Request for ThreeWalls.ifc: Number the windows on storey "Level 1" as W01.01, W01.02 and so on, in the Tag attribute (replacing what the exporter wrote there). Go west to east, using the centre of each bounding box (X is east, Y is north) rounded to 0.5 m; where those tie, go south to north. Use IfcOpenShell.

First a look at what the model holds.

```python
import ifcopenshell
import ifcopenshell.util.element
import ifcopenshell.util.placement

model = ifcopenshell.open("ThreeWalls.ifc")
print(model.schema)
storey = next(s for s in model.by_type("IfcBuildingStorey") if s.Name == "Level 1")
windows = [e for e in ifcopenshell.util.element.get_decomposition(storey) if e.is_a("IfcWindow")]
for e in sorted(windows, key=lambda e: e.id()):
    origin = ifcopenshell.util.placement.get_local_placement(e.ObjectPlacement)[:3, 3]
    print(e.id(), e.Tag, e.Name, origin.round(2) + 0.0, sep=" | ")
```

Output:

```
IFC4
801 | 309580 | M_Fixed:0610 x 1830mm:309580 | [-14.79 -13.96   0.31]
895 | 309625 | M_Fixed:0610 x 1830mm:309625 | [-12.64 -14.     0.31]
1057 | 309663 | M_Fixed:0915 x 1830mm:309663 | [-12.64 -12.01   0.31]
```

```python
import ifcopenshell
import ifcopenshell.geom
import ifcopenshell.util.element
import ifcopenshell.util.shape

model = ifcopenshell.open("ThreeWalls.ifc")
settings = ifcopenshell.geom.settings()
settings.set("use-world-coords", True)


def centre(element):
    shape = ifcopenshell.geom.create_shape(settings, element)
    return ifcopenshell.util.shape.get_bbox_centroid(shape.geometry)


storey = next(s for s in model.by_type("IfcBuildingStorey") if s.Name == "Level 1")
windows = [e for e in ifcopenshell.util.element.get_decomposition(storey) if e.is_a("IfcWindow")]

# Insertion points can sit at a corner or the storey origin, so sort by the geometry (in metres).
centres = {e: centre(e) for e in windows}
windows.sort(key=lambda e: (round(centres[e][0] / 0.5), centres[e][1]))

for i, e in enumerate(windows, start=1):
    number = f"W01.{i:02d}"
    e.Tag = number
    print(e.id(), number)

model.write("ThreeWalls_edited.ifc")
```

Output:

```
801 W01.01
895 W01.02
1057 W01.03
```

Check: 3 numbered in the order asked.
